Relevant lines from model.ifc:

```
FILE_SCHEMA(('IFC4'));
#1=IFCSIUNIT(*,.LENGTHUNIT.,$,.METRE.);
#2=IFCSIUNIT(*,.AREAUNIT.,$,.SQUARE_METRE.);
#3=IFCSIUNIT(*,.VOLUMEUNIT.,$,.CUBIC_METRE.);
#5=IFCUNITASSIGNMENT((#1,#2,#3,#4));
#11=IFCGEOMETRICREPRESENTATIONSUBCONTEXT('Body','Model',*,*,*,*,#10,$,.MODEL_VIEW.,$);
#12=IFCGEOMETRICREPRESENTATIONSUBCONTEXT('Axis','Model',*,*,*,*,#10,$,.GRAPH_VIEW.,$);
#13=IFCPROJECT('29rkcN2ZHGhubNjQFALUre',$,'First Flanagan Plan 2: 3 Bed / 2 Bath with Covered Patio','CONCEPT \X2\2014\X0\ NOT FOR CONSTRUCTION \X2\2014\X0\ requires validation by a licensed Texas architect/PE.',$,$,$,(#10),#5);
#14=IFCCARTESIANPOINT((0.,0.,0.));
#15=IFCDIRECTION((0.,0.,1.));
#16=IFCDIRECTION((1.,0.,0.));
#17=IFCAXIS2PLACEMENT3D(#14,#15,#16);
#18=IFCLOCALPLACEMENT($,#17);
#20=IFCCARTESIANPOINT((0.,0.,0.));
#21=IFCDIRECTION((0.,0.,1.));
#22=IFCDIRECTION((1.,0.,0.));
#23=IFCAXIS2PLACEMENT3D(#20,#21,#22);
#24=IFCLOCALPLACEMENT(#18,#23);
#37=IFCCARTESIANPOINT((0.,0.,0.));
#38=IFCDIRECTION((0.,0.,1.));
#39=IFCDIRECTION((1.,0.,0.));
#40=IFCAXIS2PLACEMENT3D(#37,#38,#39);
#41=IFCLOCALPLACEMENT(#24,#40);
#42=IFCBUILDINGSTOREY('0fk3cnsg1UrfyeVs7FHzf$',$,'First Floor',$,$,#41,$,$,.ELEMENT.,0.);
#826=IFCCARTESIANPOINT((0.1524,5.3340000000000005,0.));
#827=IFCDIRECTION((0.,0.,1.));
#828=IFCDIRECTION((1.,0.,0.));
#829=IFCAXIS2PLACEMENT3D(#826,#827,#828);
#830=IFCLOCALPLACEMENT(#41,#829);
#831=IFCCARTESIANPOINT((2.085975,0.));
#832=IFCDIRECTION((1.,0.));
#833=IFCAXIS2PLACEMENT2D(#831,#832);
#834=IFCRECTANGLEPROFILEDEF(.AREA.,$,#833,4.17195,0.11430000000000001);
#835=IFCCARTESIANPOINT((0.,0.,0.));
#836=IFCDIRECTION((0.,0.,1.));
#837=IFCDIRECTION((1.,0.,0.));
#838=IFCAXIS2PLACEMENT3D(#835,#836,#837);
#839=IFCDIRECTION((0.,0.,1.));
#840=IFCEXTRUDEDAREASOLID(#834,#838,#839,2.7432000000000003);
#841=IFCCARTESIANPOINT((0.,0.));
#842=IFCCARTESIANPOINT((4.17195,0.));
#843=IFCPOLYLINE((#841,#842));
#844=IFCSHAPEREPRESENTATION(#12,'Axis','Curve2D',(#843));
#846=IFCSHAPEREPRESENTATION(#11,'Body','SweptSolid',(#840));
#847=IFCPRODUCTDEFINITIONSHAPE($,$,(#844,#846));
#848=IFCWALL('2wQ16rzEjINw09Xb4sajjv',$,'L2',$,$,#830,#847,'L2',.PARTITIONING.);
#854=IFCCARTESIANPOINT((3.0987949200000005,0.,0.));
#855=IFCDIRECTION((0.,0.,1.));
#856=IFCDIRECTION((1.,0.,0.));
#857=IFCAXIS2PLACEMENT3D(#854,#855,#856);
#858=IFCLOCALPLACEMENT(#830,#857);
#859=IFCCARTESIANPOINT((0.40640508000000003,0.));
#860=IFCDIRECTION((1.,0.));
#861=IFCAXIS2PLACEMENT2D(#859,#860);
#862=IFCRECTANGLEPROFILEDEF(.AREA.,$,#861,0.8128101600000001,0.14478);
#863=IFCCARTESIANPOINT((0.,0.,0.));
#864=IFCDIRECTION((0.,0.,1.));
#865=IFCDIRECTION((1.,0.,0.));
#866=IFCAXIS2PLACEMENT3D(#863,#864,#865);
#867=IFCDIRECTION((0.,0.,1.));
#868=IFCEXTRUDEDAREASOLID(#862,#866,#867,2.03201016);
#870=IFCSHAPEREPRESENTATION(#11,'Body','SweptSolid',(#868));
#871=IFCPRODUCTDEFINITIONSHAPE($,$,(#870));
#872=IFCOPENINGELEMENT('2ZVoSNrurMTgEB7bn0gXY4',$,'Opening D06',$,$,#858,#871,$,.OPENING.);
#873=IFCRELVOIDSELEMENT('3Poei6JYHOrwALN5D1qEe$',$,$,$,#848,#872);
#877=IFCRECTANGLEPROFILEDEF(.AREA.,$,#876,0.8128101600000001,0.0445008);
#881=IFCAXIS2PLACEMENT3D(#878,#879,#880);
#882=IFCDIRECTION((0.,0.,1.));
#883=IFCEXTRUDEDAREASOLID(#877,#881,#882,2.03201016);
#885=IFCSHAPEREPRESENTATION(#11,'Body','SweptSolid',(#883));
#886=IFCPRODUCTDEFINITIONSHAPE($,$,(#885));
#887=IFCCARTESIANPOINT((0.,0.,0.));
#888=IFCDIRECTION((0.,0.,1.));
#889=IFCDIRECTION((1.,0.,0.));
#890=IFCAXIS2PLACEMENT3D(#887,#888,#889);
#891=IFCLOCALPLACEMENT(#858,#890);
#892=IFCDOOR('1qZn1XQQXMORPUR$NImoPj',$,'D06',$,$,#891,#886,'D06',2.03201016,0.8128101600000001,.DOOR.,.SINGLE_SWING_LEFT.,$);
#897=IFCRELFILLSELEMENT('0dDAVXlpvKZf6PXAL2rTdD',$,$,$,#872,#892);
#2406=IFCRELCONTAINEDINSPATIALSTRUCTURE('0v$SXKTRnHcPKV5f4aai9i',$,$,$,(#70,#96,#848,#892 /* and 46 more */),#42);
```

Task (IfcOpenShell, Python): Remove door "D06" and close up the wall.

```python
import ifcopenshell
import ifcopenshell.api.feature
import ifcopenshell.api.root
import ifcopenshell.geom
import ifcopenshell.util.shape

model = ifcopenshell.open("model.ifc")
settings = ifcopenshell.geom.settings()


def volume(element):
    """Net volume in cubic metres, openings subtracted."""
    shape = ifcopenshell.geom.create_shape(settings, element)
    return ifcopenshell.util.shape.get_volume(shape.geometry)


door = model.by_guid("1qZn1XQQXMORPUR$NImoPj")
opening = door.FillsVoids[0].RelatingOpeningElement
wall = opening.VoidsElements[0].RelatingBuildingElement
before = volume(wall)

ifcopenshell.api.root.remove_product(model, product=door)
ifcopenshell.api.feature.remove_feature(model, feature=opening)

after = volume(wall)

print(f"wall volume {before:.3f} -> {after:.3f} m3")

model.write("model_updated.ifc")
```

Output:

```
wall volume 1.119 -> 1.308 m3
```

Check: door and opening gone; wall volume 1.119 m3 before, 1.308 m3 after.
